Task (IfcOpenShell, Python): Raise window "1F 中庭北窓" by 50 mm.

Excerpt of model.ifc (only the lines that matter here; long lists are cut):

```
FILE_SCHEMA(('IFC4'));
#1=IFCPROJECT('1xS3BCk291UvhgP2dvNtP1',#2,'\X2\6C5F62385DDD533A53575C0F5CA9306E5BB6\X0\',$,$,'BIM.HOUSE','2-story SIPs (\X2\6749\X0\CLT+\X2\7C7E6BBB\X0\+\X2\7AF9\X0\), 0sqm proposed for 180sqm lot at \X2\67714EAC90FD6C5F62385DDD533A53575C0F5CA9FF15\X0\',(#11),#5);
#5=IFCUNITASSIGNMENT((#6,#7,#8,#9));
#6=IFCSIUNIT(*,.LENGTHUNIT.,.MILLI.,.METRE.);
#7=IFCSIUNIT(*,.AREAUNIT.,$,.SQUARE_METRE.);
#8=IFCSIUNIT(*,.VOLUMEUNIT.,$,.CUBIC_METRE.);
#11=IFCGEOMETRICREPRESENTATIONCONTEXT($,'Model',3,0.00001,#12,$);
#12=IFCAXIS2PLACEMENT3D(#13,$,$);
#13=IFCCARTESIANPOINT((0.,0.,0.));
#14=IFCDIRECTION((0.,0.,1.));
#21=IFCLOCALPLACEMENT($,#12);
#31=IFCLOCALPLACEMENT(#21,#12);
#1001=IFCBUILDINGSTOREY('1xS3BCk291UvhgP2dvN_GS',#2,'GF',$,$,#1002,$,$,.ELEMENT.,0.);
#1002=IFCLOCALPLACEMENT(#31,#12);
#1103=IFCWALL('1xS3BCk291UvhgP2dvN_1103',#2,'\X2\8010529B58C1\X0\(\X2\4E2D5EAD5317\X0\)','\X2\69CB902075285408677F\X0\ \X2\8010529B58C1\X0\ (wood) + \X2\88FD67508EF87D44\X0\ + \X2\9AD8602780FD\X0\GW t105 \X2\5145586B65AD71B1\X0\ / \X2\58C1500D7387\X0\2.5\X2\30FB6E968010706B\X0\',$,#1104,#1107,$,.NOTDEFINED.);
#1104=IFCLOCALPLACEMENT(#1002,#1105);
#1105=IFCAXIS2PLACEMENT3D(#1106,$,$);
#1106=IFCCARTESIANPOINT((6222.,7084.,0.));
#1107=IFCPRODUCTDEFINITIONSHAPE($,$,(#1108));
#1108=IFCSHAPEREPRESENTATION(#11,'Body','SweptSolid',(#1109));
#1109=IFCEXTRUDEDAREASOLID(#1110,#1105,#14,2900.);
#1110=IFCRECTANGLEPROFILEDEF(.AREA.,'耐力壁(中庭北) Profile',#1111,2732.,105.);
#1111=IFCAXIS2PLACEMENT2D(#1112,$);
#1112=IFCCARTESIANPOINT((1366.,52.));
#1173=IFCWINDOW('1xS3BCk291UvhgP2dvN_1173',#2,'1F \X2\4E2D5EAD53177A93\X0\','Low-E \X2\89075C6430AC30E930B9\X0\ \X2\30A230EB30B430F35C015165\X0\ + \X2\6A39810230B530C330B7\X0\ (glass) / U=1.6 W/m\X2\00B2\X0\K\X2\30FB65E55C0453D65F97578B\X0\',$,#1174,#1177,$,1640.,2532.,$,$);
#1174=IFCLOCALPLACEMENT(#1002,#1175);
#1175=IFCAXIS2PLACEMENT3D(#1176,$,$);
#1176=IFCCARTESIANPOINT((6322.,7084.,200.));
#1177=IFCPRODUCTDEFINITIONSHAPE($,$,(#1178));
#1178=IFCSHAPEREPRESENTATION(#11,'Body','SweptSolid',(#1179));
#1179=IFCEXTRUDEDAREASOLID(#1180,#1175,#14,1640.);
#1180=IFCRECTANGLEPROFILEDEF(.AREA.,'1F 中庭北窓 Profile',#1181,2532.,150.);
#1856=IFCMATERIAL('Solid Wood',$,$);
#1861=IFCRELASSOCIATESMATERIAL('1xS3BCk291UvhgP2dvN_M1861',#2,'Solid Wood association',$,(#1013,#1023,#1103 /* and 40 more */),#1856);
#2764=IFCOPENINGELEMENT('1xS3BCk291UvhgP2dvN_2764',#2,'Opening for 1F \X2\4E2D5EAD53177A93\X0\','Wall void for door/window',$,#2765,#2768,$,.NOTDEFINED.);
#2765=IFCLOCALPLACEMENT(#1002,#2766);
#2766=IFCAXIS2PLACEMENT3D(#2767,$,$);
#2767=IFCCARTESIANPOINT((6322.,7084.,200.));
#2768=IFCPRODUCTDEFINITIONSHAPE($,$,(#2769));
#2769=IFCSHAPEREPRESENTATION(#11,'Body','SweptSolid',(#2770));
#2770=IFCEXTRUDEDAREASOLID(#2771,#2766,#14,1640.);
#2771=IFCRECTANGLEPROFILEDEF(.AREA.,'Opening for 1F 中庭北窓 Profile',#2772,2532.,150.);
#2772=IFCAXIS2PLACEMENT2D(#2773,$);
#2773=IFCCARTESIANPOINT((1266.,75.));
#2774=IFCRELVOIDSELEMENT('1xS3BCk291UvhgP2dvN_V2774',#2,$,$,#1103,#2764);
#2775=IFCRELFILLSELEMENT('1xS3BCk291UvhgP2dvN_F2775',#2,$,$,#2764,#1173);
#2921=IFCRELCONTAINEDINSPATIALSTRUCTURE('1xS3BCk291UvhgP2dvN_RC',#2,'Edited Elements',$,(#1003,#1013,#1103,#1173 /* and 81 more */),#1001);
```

```python
import numpy as np
import ifcopenshell
import ifcopenshell.api.geometry
import ifcopenshell.util.placement
import ifcopenshell.util.unit

model = ifcopenshell.open("model.ifc")
unit_scale = ifcopenshell.util.unit.calculate_unit_scale(model)

window = model.by_guid("1xS3BCk291UvhgP2dvN_1173")
opening = window.FillsVoids[0].RelatingOpeningElement
dz = 0.05 / unit_scale

shift = np.array([0.0, 0.0, dz])
# The window is not placed relative to its opening, so move both.
for product in (opening, window):
    matrix = ifcopenshell.util.placement.get_local_placement(product.ObjectPlacement)
    matrix[:3, 3] += shift
    ifcopenshell.api.geometry.edit_object_placement(model, product=product, matrix=matrix, is_si=False)

print(f"moved by {dz * unit_scale:+.3f} m")

model.write("model-out.ifc")
```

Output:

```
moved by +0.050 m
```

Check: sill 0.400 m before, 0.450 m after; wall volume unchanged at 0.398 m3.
